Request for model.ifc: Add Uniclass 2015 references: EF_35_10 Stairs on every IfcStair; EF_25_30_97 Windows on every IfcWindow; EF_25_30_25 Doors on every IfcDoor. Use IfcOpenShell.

First a look at what the model holds.

```python
import ifcopenshell

model = ifcopenshell.open("model.ifc")
print(model.schema)
print("classifications:", [c.Name for c in model.by_type("IfcClassification")])
for ifc_class in ("IfcDoor", "IfcRoof", "IfcStair", "IfcWall", "IfcWindow"):
    print(ifc_class, len(model.by_type(ifc_class)))
```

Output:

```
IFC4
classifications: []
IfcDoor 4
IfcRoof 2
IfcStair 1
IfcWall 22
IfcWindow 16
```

```python
import ifcopenshell
import ifcopenshell.api.classification

model = ifcopenshell.open("model.ifc")

system = ifcopenshell.api.classification.add_classification(model, classification="Uniclass 2015")

codes = {
    "IfcStair": ("EF_35_10", "Stairs"),
    "IfcWindow": ("EF_25_30_97", "Windows"),
    "IfcDoor": ("EF_25_30_25", "Doors"),
}
for ifc_class, (code, name) in codes.items():
    products = model.by_type(ifc_class)
    ifcopenshell.api.classification.add_reference(
        model, products=products, classification=system, identification=code, name=name
    )
    print(code, len(products))

model.write("model_rev.ifc")
```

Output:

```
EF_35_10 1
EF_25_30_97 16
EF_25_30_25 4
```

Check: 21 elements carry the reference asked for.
